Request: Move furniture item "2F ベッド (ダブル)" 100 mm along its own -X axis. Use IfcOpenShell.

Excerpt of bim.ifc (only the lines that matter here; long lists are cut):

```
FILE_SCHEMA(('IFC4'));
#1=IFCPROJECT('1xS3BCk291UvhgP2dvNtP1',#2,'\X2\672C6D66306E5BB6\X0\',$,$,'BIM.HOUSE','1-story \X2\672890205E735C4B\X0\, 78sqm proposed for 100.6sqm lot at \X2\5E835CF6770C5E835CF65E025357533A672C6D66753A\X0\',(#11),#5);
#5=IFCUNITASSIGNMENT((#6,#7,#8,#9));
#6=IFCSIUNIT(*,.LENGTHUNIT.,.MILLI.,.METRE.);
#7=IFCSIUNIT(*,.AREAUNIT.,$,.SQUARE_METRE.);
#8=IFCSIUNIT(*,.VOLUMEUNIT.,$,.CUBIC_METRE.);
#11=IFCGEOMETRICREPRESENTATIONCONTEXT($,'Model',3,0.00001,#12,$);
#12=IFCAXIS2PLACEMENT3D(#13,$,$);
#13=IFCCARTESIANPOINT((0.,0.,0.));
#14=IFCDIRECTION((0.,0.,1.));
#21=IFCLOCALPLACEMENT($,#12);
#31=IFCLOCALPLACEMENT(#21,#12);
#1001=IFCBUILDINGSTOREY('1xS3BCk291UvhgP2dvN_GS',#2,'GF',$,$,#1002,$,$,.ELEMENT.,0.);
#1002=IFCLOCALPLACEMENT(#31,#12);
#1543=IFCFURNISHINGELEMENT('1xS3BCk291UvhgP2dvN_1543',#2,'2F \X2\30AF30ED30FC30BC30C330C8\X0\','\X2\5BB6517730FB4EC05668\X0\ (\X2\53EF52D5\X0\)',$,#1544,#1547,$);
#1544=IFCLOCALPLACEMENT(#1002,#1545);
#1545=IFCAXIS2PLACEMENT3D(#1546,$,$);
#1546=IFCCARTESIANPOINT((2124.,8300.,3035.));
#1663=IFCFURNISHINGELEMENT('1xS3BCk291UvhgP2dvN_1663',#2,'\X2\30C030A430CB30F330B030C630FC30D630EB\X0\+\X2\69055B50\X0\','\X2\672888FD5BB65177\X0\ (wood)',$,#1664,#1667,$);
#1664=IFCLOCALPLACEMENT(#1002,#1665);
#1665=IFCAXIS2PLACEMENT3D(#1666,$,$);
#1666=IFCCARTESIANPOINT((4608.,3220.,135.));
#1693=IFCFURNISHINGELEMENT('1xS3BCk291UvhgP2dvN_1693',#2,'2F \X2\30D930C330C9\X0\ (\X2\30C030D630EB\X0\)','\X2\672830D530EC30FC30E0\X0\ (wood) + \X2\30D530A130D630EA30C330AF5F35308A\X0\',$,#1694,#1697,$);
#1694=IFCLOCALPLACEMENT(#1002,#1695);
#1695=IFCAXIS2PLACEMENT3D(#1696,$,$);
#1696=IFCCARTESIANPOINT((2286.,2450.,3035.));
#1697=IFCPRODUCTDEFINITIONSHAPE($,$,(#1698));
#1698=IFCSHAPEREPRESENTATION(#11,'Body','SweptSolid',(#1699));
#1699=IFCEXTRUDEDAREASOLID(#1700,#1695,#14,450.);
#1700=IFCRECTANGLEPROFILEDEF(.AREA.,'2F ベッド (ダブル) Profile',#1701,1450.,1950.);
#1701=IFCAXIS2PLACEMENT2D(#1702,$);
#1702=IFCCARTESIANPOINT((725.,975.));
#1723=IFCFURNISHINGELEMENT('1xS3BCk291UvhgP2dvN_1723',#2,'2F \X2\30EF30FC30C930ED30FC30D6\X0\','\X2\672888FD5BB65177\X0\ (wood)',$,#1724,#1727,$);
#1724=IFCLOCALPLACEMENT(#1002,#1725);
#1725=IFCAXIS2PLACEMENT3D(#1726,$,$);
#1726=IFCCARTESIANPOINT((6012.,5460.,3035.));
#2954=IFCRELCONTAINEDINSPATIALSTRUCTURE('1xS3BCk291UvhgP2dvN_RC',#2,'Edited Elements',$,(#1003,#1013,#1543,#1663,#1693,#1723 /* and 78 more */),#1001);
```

```python
import ifcopenshell
import ifcopenshell.api.geometry
import ifcopenshell.util.placement
import ifcopenshell.util.unit

model = ifcopenshell.open("bim.ifc")
unit_scale = ifcopenshell.util.unit.calculate_unit_scale(model)

item = model.by_guid("1xS3BCk291UvhgP2dvN_1693")
matrix = ifcopenshell.util.placement.get_local_placement(item.ObjectPlacement)
matrix[:3, 3] -= matrix[:3, 0] * 0.1 / unit_scale
ifcopenshell.api.geometry.edit_object_placement(model, product=item, matrix=matrix, is_si=False)

print(ifcopenshell.util.placement.get_local_placement(item.ObjectPlacement).round(3) + 0.0)

model.write("bim_updated.ifc")
```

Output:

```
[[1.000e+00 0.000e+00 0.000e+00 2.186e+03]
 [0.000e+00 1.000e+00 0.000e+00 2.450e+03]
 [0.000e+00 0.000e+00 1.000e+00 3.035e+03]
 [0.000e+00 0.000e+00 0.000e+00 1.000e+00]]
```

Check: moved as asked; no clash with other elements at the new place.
